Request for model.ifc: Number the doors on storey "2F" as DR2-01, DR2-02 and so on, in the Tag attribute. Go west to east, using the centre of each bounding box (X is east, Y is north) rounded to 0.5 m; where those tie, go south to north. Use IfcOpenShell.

First a look at what the model holds.

```python
import ifcopenshell
import ifcopenshell.util.element
import ifcopenshell.util.placement

model = ifcopenshell.open("model.ifc")
print(model.schema)
storey = next(s for s in model.by_type("IfcBuildingStorey") if s.Name == "2F")
doors = [e for e in ifcopenshell.util.element.get_decomposition(storey) if e.is_a("IfcDoor")]
for e in sorted(doors, key=lambda e: e.id()):
    origin = ifcopenshell.util.placement.get_local_placement(e.ObjectPlacement)[:3, 3]
    print(e.id(), e.Tag, e.Name, origin.round(2) + 0.0, sep=" | ")
```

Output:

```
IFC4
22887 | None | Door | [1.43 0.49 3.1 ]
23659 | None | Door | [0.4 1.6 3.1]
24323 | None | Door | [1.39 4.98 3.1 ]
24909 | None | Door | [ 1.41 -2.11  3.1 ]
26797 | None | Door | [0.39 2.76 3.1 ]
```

```python
import ifcopenshell
import ifcopenshell.geom
import ifcopenshell.util.element
import ifcopenshell.util.shape

model = ifcopenshell.open("model.ifc")
settings = ifcopenshell.geom.settings()
settings.set("use-world-coords", True)


def centre(element):
    shape = ifcopenshell.geom.create_shape(settings, element)
    return ifcopenshell.util.shape.get_bbox_centroid(shape.geometry)


storey = next(s for s in model.by_type("IfcBuildingStorey") if s.Name == "2F")
doors = [e for e in ifcopenshell.util.element.get_decomposition(storey) if e.is_a("IfcDoor")]

# Insertion points can sit at a corner or the storey origin, so sort by the geometry (in metres).
centres = {e: centre(e) for e in doors}
doors.sort(key=lambda e: (round(centres[e][0] / 0.5), centres[e][1]))

for i, e in enumerate(doors, start=1):
    number = f"DR2-{i:02d}"
    e.Tag = number
    print(e.id(), number)

model.write("model_updated.ifc")
```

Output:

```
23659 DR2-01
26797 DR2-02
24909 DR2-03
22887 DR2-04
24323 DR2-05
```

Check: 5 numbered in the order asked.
